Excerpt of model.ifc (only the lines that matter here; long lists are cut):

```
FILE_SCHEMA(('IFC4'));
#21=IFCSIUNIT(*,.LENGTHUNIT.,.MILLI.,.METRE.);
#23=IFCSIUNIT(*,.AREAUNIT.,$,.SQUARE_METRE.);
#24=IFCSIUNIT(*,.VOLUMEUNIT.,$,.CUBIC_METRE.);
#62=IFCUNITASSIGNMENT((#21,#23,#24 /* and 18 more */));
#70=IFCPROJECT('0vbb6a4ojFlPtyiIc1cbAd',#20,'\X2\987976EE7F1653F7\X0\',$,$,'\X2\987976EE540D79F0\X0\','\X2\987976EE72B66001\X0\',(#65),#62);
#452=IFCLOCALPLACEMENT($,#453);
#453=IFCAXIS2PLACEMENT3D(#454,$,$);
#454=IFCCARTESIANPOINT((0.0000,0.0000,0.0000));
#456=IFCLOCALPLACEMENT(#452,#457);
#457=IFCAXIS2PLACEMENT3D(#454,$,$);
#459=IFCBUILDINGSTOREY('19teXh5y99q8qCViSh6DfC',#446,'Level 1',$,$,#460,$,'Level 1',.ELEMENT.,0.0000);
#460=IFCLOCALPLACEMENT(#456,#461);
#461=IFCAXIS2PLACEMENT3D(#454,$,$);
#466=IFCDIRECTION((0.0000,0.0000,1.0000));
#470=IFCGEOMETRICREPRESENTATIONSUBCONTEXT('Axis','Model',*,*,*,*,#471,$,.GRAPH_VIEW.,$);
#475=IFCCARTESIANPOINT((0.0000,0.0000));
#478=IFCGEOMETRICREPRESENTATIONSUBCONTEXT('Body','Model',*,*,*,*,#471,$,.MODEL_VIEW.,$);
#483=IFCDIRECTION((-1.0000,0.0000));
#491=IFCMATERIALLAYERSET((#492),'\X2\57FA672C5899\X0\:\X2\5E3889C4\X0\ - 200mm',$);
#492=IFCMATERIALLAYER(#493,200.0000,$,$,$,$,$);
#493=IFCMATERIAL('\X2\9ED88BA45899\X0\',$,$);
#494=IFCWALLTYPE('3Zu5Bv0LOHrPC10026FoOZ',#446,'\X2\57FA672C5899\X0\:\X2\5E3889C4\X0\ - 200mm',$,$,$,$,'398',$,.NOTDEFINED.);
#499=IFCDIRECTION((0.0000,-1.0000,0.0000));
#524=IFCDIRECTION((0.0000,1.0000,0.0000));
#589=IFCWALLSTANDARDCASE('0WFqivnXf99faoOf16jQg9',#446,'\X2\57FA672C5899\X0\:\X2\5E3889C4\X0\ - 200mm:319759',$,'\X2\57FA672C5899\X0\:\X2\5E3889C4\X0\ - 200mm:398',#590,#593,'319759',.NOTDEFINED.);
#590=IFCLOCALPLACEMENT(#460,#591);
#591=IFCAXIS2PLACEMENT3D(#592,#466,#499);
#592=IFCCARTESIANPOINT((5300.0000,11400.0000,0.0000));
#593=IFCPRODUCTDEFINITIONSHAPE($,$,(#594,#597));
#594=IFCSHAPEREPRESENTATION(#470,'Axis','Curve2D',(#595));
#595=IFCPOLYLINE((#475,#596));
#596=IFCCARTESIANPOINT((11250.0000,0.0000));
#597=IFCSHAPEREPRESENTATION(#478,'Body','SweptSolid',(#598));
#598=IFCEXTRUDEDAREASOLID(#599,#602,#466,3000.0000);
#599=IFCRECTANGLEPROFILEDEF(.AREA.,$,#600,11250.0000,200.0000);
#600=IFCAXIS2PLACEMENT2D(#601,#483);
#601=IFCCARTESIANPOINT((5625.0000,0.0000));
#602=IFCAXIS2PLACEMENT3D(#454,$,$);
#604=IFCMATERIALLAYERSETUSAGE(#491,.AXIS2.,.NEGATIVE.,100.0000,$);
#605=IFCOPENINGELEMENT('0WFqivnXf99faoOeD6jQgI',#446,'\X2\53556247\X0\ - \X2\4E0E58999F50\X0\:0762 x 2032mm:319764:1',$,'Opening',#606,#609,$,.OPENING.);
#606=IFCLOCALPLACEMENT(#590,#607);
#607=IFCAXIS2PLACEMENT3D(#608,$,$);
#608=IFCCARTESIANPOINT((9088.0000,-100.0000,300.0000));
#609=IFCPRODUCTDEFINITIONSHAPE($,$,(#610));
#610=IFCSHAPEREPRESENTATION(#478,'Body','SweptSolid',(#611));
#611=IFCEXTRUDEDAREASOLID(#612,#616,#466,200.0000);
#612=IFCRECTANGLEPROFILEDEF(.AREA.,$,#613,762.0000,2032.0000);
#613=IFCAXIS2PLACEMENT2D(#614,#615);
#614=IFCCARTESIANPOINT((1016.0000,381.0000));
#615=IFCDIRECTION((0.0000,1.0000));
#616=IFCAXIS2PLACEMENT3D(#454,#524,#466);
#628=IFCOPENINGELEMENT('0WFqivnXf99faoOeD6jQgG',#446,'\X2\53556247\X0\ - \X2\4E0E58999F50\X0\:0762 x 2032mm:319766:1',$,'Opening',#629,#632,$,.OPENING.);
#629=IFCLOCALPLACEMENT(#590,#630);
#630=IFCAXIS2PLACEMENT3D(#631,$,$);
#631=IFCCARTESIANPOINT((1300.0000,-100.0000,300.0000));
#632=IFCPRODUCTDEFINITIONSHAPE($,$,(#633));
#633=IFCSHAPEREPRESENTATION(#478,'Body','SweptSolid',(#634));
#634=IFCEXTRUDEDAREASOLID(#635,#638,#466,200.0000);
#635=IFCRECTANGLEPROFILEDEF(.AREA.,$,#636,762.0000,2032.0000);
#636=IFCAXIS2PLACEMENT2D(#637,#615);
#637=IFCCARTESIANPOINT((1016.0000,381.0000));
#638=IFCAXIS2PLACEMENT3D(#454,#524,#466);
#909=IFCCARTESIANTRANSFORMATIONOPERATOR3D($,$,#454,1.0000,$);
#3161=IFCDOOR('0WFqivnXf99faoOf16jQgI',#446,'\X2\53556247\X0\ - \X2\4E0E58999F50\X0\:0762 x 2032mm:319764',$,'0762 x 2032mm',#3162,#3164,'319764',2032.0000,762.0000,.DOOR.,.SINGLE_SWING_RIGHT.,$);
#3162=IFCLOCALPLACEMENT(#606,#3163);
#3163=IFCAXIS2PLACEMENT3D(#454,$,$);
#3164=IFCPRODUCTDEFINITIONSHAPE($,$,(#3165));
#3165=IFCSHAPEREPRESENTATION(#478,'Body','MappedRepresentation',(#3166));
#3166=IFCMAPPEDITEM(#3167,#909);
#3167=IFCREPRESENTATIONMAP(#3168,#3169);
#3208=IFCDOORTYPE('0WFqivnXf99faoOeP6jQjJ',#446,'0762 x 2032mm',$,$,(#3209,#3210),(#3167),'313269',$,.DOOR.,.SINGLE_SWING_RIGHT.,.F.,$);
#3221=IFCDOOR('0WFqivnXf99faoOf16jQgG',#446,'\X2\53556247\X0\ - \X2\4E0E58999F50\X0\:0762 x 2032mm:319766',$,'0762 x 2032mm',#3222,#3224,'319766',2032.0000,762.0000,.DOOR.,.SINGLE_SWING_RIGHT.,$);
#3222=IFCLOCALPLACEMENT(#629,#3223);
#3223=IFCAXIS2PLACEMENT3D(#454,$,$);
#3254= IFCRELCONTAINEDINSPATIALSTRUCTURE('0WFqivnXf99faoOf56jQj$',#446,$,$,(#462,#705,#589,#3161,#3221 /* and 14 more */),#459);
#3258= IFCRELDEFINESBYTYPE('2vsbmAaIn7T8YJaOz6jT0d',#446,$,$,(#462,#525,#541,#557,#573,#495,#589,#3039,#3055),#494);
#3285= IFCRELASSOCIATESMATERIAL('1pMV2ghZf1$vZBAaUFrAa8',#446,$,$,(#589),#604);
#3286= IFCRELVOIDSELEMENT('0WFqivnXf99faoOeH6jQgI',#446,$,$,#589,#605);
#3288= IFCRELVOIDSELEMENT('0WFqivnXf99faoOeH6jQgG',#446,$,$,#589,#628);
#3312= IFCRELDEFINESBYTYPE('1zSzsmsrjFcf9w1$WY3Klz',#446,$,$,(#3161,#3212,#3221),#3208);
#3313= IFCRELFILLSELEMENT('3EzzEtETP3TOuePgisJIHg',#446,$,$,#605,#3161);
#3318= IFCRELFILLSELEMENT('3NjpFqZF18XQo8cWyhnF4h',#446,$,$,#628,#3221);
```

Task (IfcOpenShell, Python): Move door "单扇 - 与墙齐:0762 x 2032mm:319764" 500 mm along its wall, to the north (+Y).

```python
import ifcopenshell
import ifcopenshell.api.geometry
import ifcopenshell.util.placement

model = ifcopenshell.open("model.ifc")

door = model.by_guid("0WFqivnXf99faoOf16jQgI")
opening = door.FillsVoids[0].RelatingOpeningElement
wall = opening.VoidsElements[0].RelatingBuildingElement

wall_matrix = ifcopenshell.util.placement.get_local_placement(wall.ObjectPlacement)
shift = wall_matrix[:3, 0] * -500.0
before = ifcopenshell.util.placement.get_local_placement(door.ObjectPlacement)[:3, 3].copy()

# The door is placed relative to its opening, so it follows when the opening moves.
matrix = ifcopenshell.util.placement.get_local_placement(opening.ObjectPlacement)
matrix[:3, 3] += shift
ifcopenshell.api.geometry.edit_object_placement(
    model, product=opening, matrix=matrix, is_si=False, should_transform_children=True
)

after = ifcopenshell.util.placement.get_local_placement(door.ObjectPlacement)[:3, 3]
print("door moved by", (after - before).round(3) + 0.0)

model.write("model-out.ifc")
```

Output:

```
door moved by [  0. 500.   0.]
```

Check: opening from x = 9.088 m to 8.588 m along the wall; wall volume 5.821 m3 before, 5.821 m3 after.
